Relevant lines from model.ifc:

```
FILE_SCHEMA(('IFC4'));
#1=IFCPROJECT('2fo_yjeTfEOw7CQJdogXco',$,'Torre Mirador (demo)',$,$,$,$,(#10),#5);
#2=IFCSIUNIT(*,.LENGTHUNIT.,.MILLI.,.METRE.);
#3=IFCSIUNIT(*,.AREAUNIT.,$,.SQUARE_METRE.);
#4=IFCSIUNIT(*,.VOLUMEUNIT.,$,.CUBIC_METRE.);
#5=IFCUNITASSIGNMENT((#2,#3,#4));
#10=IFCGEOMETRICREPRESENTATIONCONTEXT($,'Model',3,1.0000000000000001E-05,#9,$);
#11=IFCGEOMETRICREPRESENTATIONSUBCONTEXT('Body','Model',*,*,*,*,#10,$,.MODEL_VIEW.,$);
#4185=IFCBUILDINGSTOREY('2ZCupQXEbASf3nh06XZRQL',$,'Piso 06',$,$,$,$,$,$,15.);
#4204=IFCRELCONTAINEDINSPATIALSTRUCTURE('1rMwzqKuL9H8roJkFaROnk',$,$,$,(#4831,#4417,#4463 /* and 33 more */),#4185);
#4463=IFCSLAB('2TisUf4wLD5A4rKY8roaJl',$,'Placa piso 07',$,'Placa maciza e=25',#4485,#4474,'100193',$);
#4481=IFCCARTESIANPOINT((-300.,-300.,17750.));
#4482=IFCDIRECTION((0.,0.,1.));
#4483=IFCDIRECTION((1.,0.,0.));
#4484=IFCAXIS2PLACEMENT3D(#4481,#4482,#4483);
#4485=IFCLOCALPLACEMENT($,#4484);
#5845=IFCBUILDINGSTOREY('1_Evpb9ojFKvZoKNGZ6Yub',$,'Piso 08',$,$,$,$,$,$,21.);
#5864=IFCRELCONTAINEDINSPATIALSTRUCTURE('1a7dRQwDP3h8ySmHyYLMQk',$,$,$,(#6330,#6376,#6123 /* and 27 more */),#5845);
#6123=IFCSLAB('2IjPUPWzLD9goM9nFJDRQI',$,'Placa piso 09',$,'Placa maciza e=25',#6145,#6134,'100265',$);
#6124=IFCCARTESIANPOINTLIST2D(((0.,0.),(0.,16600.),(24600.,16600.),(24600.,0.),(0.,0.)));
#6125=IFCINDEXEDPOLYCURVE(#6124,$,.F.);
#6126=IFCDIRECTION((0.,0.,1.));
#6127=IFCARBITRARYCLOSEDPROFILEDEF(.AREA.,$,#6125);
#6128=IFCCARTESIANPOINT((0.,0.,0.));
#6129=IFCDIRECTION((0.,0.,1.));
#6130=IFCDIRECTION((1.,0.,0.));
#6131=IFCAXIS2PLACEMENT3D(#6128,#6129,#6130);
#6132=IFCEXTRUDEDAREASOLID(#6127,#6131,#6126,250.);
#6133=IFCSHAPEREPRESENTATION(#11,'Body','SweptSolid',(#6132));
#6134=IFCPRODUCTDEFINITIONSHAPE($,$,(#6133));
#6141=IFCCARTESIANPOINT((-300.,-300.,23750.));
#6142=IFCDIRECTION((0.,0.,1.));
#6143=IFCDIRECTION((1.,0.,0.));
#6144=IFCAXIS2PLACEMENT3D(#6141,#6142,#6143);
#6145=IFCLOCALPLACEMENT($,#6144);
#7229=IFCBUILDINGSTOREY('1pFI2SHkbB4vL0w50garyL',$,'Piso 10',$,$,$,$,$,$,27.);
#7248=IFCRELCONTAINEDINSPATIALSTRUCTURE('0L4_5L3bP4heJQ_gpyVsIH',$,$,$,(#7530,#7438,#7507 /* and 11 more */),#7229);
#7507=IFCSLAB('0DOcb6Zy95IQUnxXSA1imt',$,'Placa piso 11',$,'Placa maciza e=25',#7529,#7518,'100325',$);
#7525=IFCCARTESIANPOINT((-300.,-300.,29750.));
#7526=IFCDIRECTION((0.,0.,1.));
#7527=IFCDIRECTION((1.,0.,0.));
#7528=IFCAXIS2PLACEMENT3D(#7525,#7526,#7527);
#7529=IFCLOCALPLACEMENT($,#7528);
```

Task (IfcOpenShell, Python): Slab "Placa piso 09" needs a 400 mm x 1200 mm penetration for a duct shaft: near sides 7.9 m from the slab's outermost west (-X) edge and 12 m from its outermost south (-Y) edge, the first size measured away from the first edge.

```python
import numpy as np
import ifcopenshell
import ifcopenshell.api.feature
import ifcopenshell.api.geometry
import ifcopenshell.api.root
import ifcopenshell.geom
import ifcopenshell.util.placement
import ifcopenshell.util.representation
import ifcopenshell.util.shape
import ifcopenshell.util.unit

model = ifcopenshell.open("model.ifc")
unit_scale = ifcopenshell.util.unit.calculate_unit_scale(model)
settings = ifcopenshell.geom.settings()


def volume(element):
    """Net volume in cubic metres, openings subtracted."""
    shape = ifcopenshell.geom.create_shape(settings, element)
    return ifcopenshell.util.shape.get_volume(shape.geometry)


slab = model.by_guid("2IjPUPWzLD9goM9nFJDRQI")
before = volume(slab)

# Extent in the slab's own axes, in metres. The edges named are its -X and -Y sides.
slab_shape = ifcopenshell.geom.create_shape(settings, slab)
vertices = ifcopenshell.util.shape.get_vertices(slab_shape.geometry)
x_min, y_min, bottom = vertices.min(axis=0)
top = vertices[:, 2].max()

opening = ifcopenshell.api.root.create_entity(model, ifc_class="IfcOpeningElement", name="Duct shaft opening", predefined_type="OPENING")
context = ifcopenshell.util.representation.get_context(model, "Model", "Body", "MODEL_VIEW")
width, depth = 0.4, 1.2
outline = [(0.0, 0.0), (width, 0.0), (width, depth), (0.0, depth), (0.0, 0.0)]
# Overshoot both faces by 50 mm so the cut is clean.
shape = ifcopenshell.api.geometry.add_slab_representation(
    model, context=context, depth=top - bottom + 0.1, polyline=outline
)
ifcopenshell.api.geometry.assign_representation(model, product=opening, representation=shape)

matrix = ifcopenshell.util.placement.get_local_placement(slab.ObjectPlacement)
matrix[:, 3] = matrix @ np.append(np.array([x_min + 7.9, y_min + 12, bottom - 0.05]) / unit_scale, 1.0)
ifcopenshell.api.geometry.edit_object_placement(model, product=opening, matrix=matrix, is_si=False)
ifcopenshell.api.feature.add_feature(model, feature=opening, element=slab)

after = volume(slab)

print(f"slab volume {before:.3f} -> {after:.3f} m3")

model.write("model_rev.ifc")
```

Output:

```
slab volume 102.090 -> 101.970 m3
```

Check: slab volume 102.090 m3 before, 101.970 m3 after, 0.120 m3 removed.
